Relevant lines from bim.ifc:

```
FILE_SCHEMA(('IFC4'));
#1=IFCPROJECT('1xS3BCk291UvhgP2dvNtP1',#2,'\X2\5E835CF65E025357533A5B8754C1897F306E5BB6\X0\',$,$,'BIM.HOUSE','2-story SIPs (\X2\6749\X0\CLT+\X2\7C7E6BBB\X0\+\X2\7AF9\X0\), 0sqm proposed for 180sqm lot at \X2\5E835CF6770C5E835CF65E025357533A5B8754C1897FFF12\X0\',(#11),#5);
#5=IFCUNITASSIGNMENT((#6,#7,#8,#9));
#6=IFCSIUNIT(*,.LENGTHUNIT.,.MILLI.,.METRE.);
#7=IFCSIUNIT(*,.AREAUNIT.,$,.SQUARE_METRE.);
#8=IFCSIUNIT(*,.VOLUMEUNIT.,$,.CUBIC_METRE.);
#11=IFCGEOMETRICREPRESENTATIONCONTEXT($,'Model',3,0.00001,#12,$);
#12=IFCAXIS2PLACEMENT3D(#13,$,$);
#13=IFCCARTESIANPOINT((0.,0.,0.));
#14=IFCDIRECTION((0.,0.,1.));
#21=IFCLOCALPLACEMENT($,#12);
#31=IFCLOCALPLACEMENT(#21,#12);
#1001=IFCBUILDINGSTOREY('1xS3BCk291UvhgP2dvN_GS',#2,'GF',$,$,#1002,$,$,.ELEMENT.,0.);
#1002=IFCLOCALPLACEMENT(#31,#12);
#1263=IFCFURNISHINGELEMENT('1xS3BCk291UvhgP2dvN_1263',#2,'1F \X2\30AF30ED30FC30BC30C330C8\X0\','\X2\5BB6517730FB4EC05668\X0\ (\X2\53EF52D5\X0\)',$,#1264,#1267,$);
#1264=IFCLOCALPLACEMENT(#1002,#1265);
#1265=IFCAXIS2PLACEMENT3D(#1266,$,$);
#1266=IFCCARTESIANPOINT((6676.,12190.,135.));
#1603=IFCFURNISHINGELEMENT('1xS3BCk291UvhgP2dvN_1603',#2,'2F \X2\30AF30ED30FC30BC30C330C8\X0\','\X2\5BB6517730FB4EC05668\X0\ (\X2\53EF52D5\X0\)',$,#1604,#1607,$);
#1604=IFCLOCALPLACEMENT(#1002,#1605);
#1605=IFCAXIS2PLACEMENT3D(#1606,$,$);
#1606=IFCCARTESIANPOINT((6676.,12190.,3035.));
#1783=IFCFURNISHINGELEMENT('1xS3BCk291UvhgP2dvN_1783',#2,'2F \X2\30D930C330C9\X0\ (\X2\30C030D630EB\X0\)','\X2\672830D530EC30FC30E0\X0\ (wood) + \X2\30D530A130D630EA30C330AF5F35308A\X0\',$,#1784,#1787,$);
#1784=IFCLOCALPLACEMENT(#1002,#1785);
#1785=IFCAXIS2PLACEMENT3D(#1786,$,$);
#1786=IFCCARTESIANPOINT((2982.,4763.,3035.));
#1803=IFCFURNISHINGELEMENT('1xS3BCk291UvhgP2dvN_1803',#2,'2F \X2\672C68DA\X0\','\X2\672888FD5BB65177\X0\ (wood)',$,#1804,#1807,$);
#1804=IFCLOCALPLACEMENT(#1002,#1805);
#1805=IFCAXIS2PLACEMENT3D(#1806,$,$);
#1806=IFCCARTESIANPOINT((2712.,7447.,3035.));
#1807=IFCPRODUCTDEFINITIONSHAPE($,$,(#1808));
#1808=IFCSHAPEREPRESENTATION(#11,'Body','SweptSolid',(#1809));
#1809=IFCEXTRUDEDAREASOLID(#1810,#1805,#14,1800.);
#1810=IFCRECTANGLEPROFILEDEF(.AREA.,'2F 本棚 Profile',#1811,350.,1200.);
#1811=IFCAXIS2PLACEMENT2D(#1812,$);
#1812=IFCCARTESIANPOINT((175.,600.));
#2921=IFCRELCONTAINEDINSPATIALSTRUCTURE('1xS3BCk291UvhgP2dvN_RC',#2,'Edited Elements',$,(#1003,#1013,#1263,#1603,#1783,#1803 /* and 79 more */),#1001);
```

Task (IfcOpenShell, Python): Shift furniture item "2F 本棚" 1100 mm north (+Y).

```python
import ifcopenshell
import ifcopenshell.api.geometry
import ifcopenshell.util.placement

model = ifcopenshell.open("bim.ifc")

item = model.by_id(1803)
matrix = ifcopenshell.util.placement.get_local_placement(item.ObjectPlacement)
matrix[1, 3] += 1100.0
ifcopenshell.api.geometry.edit_object_placement(model, product=item, matrix=matrix, is_si=False)

print(ifcopenshell.util.placement.get_local_placement(item.ObjectPlacement).round(3) + 0.0)

model.write("bim-out.ifc")
```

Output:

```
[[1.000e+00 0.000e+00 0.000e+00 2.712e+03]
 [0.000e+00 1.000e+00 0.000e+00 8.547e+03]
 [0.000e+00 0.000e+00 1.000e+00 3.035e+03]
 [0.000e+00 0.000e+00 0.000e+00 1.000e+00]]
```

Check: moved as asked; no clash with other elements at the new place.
